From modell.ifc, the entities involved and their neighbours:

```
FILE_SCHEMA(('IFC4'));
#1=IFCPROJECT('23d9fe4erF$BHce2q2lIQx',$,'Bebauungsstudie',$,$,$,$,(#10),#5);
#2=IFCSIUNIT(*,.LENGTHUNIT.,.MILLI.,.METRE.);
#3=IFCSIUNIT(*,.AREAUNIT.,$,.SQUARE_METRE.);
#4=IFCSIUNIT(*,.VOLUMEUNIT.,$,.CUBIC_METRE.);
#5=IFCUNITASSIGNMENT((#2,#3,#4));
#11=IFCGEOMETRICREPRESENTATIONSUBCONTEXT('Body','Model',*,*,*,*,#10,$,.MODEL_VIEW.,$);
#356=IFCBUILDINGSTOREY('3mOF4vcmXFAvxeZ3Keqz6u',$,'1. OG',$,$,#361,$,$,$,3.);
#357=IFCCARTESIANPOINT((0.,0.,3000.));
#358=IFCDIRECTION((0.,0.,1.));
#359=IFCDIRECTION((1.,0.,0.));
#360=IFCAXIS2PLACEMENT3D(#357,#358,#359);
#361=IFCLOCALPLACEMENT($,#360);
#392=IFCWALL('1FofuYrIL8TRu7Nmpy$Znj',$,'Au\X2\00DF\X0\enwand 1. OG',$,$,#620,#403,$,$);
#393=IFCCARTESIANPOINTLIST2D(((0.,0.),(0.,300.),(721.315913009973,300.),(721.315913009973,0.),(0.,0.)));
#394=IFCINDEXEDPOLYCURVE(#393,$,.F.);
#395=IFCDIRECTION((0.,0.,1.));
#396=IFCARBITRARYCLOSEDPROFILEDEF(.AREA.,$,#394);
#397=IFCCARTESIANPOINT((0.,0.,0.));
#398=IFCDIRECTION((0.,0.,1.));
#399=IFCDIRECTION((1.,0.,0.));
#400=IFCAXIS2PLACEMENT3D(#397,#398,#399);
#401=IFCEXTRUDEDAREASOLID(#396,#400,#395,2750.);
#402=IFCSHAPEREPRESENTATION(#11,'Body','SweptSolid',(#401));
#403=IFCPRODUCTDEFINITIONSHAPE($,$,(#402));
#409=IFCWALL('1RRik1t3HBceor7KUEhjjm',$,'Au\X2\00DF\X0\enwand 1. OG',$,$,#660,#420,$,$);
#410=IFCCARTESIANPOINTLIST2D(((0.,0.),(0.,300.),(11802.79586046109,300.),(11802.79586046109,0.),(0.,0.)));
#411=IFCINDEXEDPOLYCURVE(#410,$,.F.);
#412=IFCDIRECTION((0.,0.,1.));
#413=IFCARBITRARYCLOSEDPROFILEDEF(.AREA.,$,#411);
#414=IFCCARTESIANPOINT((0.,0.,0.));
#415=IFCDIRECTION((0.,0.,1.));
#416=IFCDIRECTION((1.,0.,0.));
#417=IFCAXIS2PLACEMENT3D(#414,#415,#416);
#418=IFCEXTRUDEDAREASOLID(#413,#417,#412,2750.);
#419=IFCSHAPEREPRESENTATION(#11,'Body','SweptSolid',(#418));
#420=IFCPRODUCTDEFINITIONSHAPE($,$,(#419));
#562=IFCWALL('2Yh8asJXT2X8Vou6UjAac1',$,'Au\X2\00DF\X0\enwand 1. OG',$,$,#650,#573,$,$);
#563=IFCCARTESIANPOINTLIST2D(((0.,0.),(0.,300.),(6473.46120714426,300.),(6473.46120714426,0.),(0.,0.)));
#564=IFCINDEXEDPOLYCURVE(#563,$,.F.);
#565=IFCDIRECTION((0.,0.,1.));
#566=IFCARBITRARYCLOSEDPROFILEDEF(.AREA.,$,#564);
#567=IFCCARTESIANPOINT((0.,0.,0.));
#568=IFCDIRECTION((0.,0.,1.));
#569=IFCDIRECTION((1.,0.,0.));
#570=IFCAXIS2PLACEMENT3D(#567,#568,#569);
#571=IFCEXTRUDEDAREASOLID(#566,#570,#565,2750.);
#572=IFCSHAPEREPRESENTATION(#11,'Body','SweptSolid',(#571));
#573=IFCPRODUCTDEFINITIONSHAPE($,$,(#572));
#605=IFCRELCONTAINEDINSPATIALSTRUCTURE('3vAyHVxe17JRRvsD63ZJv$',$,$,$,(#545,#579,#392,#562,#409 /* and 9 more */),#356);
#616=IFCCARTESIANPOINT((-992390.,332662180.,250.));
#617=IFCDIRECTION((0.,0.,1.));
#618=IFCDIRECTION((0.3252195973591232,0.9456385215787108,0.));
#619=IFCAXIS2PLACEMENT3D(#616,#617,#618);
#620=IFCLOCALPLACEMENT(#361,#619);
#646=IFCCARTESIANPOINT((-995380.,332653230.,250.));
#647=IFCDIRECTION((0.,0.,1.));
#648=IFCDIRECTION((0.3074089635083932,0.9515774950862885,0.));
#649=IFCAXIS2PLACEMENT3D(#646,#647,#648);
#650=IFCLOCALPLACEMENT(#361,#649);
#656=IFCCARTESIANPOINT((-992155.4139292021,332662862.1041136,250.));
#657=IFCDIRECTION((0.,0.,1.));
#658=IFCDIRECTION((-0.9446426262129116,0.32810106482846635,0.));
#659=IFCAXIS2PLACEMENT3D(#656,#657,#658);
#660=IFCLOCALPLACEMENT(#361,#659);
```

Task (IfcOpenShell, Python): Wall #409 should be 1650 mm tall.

```python
import ifcopenshell
import ifcopenshell.geom
import ifcopenshell.util.representation
import ifcopenshell.util.shape
import ifcopenshell.util.unit

model = ifcopenshell.open("modell.ifc")
unit_scale = ifcopenshell.util.unit.calculate_unit_scale(model)
settings = ifcopenshell.geom.settings()


def volume(element):
    """Net volume in cubic metres, openings subtracted."""
    shape = ifcopenshell.geom.create_shape(settings, element)
    return ifcopenshell.util.shape.get_volume(shape.geometry)


wall = model.by_guid("1RRik1t3HBceor7KUEhjjm")
before = volume(wall)

body = ifcopenshell.util.representation.get_representation(wall, "Model", "Body")
solid = body.Items[0]
old_height = solid.Depth
solid.Depth = 1.65 / unit_scale
after = volume(wall)

print(f"height {old_height:g} -> {solid.Depth:g}, volume {before:.3f} -> {after:.3f} m3")

model.write("modell-out.ifc")
```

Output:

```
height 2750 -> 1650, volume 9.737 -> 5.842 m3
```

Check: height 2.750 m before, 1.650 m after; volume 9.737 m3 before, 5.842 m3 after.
